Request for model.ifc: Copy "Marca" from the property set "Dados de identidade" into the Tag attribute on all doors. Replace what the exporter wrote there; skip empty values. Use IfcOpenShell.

First a look at what the model holds.

```python
import ifcopenshell
import ifcopenshell.util.element

model = ifcopenshell.open("model.ifc")
print(model.schema)
doors = model.by_type("IfcDoor")
print(len(doors), "doors")
for e in doors[:8]:
    source = ifcopenshell.util.element.get_pset(e, "Dados de identidade", "Marca")
    target = e.Tag
    print(e.id(), repr(source), repr(target), sep=" | ")
```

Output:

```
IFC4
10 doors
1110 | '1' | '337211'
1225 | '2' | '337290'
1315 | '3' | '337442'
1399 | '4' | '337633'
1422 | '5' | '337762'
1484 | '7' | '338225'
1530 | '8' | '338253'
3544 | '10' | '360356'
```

```python
import ifcopenshell
import ifcopenshell.util.element

model = ifcopenshell.open("model.ifc")

count = 0
for e in model.by_type("IfcDoor"):
    value = ifcopenshell.util.element.get_pset(e, "Dados de identidade", "Marca")
    current = e.Tag
    if not value or not value.strip() or current == value:
        continue
    e.Tag = value
    count += 1

print(count, "doors updated")

model.write("model-out.ifc")
```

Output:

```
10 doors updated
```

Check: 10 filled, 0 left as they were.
